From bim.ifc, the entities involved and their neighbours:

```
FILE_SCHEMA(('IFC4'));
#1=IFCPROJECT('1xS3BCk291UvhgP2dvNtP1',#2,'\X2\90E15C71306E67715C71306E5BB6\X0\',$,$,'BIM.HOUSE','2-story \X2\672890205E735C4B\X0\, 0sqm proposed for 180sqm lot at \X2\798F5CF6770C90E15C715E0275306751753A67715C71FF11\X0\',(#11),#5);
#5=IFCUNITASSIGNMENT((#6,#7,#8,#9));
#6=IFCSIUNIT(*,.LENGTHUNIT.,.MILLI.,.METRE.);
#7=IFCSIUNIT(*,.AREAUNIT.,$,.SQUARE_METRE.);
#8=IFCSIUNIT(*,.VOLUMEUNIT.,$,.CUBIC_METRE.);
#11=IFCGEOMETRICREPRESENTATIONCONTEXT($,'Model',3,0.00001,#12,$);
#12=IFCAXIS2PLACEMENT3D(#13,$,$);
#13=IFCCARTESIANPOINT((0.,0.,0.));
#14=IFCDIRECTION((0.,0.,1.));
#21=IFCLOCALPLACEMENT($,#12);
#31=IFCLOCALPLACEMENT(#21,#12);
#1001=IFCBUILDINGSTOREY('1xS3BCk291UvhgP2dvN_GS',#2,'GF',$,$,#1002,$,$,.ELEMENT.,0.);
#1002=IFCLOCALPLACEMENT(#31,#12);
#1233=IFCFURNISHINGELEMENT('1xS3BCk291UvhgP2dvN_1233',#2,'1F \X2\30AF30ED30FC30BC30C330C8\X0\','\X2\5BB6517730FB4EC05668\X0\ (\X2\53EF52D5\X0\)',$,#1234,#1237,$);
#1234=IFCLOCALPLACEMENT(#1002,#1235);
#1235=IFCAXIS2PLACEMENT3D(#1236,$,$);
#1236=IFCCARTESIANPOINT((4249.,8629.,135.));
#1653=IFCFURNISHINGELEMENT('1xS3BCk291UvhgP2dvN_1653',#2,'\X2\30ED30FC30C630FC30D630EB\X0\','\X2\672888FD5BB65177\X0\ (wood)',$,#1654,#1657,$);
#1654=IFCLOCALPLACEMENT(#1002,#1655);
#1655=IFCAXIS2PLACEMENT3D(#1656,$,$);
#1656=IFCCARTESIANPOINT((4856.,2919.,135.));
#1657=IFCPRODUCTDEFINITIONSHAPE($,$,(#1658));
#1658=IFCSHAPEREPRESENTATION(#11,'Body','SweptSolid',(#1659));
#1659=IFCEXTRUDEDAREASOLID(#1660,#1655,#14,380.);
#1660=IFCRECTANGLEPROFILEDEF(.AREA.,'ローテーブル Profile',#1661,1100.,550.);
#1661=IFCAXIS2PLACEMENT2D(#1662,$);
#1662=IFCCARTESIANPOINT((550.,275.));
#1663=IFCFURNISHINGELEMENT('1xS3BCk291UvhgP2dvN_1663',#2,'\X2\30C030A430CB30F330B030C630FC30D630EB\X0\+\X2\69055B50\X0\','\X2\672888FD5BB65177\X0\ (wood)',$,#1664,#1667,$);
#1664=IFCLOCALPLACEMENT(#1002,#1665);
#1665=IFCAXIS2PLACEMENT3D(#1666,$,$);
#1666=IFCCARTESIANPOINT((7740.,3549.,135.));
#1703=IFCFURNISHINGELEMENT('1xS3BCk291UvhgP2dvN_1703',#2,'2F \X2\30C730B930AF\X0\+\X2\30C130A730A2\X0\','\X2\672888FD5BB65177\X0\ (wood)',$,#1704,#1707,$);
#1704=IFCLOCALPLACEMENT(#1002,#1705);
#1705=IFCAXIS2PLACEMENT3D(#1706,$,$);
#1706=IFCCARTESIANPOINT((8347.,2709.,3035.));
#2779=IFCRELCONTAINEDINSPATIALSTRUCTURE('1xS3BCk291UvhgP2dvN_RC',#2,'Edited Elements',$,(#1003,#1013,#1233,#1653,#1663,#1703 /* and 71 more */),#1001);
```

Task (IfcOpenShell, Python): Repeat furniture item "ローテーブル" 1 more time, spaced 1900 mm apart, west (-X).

```python
import numpy as np
import ifcopenshell
import ifcopenshell.api.geometry
import ifcopenshell.api.root
import ifcopenshell.util.element
import ifcopenshell.util.placement

model = ifcopenshell.open("bim.ifc")


def reuse_history(source, copy):
    """copy_class also copies each property set's owner history, people and application; keep the originals."""
    for rel in copy.IsDefinedBy:
        if rel.is_a("IfcRelDefinesByProperties") and (history := rel.RelatingPropertyDefinition.OwnerHistory):
            rel.RelatingPropertyDefinition.OwnerHistory = source.OwnerHistory
            ifcopenshell.util.element.remove_deep2(model, history)


source = model.by_guid("1xS3BCk291UvhgP2dvN_1653")
base = ifcopenshell.util.placement.get_local_placement(source.ObjectPlacement)
step = np.array([-1.0, 0.0, 0.0]) * 1900.0

for i in range(1, 2):
    copy = ifcopenshell.api.root.copy_class(model, product=source)
    copy.Representation = ifcopenshell.util.element.copy_deep(
        model, source.Representation, exclude=["IfcGeometricRepresentationContext", "IfcRepresentationMap"]
    )
    reuse_history(source, copy)
    matrix = base.copy()
    matrix[:3, 3] += i * step
    print("added at", matrix[:3, 3].round(3) + 0.0)
    ifcopenshell.api.geometry.edit_object_placement(model, product=copy, matrix=matrix, is_si=False)

model.write("bim_updated.ifc")
```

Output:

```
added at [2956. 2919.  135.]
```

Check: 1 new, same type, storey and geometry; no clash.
